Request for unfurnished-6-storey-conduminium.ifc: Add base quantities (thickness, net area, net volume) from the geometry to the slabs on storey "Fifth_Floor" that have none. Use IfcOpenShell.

First a look at what the model holds.

```python
import ifcopenshell
import ifcopenshell.util.element
import ifcopenshell.util.unit

model = ifcopenshell.open("unfurnished-6-storey-conduminium.ifc")
print(model.schema)
for unit_type in ("LENGTHUNIT", "AREAUNIT", "VOLUMEUNIT"):
    print(unit_type, ifcopenshell.util.unit.calculate_unit_scale(model, unit_type))
storey = next(s for s in model.by_type("IfcBuildingStorey") if s.Name == "Fifth_Floor")
slabs = [e for e in ifcopenshell.util.element.get_decomposition(storey) if e.is_a("IfcSlab")]
for e in sorted(slabs, key=lambda e: e.id()):
    print(e.id(), e.is_a(), e.Name, list(ifcopenshell.util.element.get_psets(e, qtos_only=True)), sep=" | ")
```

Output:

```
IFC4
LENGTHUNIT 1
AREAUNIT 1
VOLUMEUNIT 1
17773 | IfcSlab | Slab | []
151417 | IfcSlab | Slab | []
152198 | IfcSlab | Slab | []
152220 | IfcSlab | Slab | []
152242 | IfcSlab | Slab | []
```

```python
import ifcopenshell
import ifcopenshell.api.pset
import ifcopenshell.geom
import ifcopenshell.util.element
import ifcopenshell.util.shape
import ifcopenshell.util.unit

model = ifcopenshell.open("unfurnished-6-storey-conduminium.ifc")
unit_scale = ifcopenshell.util.unit.calculate_unit_scale(model)
area_scale = ifcopenshell.util.unit.calculate_unit_scale(model, "AREAUNIT")
volume_scale = ifcopenshell.util.unit.calculate_unit_scale(model, "VOLUMEUNIT")
settings = ifcopenshell.geom.settings()

storey = next(s for s in model.by_type("IfcBuildingStorey") if s.Name == "Fifth_Floor")
slabs = [e for e in ifcopenshell.util.element.get_decomposition(storey) if e.is_a("IfcSlab")]

for e in sorted(slabs, key=lambda e: e.id()):
    if ifcopenshell.util.element.get_psets(e, qtos_only=True, should_inherit=False):
        continue
    # Geometry comes back in metres, in the element's own axes.
    shape = ifcopenshell.geom.create_shape(settings, e)
    values = {
        "Width": ifcopenshell.util.shape.get_z(shape.geometry) / unit_scale,
        "NetArea": ifcopenshell.util.shape.get_footprint_area(shape.geometry) / area_scale,
        "NetVolume": ifcopenshell.util.shape.get_volume(shape.geometry) / volume_scale,
    }
    qto = ifcopenshell.api.pset.add_qto(model, product=e, name="Qto_SlabBaseQuantities")
    ifcopenshell.api.pset.edit_qto(model, qto=qto, properties=values)
    print(e.id(), {k: round(v, 3) for k, v in values.items()})

model.write("unfurnished-6-storey-conduminium_rev.ifc")
```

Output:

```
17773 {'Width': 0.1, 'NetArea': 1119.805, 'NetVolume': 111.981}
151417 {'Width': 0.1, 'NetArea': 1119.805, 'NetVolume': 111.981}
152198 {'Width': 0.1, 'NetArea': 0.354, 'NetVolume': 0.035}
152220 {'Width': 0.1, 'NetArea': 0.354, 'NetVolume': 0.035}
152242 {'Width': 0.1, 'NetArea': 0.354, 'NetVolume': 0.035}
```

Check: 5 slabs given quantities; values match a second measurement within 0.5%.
